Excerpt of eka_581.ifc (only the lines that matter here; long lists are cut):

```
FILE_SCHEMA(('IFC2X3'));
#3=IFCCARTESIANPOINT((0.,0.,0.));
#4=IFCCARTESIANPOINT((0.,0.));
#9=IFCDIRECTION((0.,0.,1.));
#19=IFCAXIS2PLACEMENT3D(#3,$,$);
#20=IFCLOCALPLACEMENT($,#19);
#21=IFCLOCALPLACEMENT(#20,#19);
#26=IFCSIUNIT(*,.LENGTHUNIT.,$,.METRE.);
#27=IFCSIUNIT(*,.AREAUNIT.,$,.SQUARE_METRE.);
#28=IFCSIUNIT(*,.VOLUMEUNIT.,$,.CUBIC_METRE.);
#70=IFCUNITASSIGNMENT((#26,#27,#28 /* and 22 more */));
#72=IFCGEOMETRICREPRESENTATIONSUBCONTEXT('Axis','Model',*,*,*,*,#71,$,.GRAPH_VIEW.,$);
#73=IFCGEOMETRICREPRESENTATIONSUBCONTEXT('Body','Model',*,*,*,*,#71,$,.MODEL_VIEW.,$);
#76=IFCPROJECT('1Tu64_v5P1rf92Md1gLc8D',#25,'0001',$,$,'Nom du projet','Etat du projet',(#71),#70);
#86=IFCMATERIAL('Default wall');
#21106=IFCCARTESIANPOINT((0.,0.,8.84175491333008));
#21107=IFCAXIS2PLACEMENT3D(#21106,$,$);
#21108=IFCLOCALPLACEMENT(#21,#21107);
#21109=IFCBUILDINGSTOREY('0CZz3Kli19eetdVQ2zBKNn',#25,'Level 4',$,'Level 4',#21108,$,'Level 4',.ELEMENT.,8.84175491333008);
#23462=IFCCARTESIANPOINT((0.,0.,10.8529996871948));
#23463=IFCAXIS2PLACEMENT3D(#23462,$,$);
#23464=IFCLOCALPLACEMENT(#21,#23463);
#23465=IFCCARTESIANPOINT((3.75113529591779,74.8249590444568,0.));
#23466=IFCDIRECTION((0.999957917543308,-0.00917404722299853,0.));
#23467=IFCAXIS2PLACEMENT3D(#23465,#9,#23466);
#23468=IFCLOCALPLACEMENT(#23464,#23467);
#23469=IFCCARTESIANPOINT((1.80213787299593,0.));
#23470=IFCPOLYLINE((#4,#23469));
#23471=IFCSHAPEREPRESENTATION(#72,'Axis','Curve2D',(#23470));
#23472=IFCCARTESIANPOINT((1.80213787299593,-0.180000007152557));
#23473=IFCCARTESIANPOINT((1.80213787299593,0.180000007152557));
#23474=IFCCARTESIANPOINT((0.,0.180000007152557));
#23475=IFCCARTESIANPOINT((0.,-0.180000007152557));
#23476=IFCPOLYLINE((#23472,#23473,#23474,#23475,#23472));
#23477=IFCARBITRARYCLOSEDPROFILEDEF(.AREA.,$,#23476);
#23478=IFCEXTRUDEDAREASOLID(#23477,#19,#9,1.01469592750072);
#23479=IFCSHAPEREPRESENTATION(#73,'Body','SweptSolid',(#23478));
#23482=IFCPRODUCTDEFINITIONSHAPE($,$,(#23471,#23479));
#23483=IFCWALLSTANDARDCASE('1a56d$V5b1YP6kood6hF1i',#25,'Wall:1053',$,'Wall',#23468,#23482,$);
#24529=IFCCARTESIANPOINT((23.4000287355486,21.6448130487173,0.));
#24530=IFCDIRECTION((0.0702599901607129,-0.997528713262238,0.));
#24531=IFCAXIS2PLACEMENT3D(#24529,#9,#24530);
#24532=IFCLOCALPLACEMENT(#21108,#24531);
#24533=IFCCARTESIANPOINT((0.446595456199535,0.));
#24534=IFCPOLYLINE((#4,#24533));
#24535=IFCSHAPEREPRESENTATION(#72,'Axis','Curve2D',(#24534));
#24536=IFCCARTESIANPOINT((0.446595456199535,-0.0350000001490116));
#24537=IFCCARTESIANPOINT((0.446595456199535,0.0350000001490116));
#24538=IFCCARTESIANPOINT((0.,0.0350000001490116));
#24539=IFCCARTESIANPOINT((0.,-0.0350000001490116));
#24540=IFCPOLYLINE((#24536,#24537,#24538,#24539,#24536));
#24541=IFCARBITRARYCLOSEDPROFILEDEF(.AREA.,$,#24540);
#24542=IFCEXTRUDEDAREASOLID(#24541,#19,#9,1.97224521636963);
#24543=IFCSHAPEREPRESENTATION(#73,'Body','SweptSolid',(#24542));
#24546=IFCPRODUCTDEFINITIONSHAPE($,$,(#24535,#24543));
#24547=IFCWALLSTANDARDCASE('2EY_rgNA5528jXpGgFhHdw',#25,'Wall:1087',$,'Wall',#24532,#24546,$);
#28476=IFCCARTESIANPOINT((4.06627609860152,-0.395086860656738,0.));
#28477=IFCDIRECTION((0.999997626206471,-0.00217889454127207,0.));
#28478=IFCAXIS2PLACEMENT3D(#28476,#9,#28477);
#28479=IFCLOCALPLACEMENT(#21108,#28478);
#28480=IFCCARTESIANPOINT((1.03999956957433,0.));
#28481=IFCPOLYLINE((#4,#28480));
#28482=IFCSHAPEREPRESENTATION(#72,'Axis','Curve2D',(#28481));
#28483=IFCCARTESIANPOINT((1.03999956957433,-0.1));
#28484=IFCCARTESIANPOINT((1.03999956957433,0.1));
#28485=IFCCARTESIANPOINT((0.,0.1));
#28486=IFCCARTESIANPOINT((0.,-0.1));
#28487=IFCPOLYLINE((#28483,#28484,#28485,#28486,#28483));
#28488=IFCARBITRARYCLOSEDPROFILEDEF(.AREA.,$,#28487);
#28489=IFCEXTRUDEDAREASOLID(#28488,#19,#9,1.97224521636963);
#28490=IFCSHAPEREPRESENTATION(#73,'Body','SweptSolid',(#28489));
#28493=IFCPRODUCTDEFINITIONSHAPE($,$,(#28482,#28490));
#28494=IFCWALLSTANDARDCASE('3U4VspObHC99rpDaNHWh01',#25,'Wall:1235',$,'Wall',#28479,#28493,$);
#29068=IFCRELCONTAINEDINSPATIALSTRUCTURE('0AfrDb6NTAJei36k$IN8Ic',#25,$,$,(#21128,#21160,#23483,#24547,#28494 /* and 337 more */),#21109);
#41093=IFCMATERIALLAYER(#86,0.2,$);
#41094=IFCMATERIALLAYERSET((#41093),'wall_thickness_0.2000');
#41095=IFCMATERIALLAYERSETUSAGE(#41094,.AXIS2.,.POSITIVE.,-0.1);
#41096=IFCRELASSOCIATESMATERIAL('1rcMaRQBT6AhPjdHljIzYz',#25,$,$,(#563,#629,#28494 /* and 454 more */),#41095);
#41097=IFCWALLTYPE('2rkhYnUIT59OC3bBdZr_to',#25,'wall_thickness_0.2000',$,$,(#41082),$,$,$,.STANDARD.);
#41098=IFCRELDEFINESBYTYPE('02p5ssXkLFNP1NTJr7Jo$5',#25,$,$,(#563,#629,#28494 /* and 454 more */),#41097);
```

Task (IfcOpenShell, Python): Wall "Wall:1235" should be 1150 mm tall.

```python
import ifcopenshell
import ifcopenshell.geom
import ifcopenshell.util.representation
import ifcopenshell.util.shape
import ifcopenshell.util.unit

model = ifcopenshell.open("eka_581.ifc")
unit_scale = ifcopenshell.util.unit.calculate_unit_scale(model)
settings = ifcopenshell.geom.settings()


def volume(element):
    """Net volume in cubic metres, openings subtracted."""
    shape = ifcopenshell.geom.create_shape(settings, element)
    return ifcopenshell.util.shape.get_volume(shape.geometry)


wall = model.by_guid("3U4VspObHC99rpDaNHWh01")
before = volume(wall)

body = ifcopenshell.util.representation.get_representation(wall, "Model", "Body")
solid = body.Items[0]
old_height = solid.Depth
solid.Depth = 1.15 / unit_scale
after = volume(wall)

print(f"height {old_height:g} -> {solid.Depth:g}, volume {before:.3f} -> {after:.3f} m3")

model.write("eka_581_rev.ifc")
```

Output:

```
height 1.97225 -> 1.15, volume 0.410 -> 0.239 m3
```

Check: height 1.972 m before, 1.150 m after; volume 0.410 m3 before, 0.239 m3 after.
